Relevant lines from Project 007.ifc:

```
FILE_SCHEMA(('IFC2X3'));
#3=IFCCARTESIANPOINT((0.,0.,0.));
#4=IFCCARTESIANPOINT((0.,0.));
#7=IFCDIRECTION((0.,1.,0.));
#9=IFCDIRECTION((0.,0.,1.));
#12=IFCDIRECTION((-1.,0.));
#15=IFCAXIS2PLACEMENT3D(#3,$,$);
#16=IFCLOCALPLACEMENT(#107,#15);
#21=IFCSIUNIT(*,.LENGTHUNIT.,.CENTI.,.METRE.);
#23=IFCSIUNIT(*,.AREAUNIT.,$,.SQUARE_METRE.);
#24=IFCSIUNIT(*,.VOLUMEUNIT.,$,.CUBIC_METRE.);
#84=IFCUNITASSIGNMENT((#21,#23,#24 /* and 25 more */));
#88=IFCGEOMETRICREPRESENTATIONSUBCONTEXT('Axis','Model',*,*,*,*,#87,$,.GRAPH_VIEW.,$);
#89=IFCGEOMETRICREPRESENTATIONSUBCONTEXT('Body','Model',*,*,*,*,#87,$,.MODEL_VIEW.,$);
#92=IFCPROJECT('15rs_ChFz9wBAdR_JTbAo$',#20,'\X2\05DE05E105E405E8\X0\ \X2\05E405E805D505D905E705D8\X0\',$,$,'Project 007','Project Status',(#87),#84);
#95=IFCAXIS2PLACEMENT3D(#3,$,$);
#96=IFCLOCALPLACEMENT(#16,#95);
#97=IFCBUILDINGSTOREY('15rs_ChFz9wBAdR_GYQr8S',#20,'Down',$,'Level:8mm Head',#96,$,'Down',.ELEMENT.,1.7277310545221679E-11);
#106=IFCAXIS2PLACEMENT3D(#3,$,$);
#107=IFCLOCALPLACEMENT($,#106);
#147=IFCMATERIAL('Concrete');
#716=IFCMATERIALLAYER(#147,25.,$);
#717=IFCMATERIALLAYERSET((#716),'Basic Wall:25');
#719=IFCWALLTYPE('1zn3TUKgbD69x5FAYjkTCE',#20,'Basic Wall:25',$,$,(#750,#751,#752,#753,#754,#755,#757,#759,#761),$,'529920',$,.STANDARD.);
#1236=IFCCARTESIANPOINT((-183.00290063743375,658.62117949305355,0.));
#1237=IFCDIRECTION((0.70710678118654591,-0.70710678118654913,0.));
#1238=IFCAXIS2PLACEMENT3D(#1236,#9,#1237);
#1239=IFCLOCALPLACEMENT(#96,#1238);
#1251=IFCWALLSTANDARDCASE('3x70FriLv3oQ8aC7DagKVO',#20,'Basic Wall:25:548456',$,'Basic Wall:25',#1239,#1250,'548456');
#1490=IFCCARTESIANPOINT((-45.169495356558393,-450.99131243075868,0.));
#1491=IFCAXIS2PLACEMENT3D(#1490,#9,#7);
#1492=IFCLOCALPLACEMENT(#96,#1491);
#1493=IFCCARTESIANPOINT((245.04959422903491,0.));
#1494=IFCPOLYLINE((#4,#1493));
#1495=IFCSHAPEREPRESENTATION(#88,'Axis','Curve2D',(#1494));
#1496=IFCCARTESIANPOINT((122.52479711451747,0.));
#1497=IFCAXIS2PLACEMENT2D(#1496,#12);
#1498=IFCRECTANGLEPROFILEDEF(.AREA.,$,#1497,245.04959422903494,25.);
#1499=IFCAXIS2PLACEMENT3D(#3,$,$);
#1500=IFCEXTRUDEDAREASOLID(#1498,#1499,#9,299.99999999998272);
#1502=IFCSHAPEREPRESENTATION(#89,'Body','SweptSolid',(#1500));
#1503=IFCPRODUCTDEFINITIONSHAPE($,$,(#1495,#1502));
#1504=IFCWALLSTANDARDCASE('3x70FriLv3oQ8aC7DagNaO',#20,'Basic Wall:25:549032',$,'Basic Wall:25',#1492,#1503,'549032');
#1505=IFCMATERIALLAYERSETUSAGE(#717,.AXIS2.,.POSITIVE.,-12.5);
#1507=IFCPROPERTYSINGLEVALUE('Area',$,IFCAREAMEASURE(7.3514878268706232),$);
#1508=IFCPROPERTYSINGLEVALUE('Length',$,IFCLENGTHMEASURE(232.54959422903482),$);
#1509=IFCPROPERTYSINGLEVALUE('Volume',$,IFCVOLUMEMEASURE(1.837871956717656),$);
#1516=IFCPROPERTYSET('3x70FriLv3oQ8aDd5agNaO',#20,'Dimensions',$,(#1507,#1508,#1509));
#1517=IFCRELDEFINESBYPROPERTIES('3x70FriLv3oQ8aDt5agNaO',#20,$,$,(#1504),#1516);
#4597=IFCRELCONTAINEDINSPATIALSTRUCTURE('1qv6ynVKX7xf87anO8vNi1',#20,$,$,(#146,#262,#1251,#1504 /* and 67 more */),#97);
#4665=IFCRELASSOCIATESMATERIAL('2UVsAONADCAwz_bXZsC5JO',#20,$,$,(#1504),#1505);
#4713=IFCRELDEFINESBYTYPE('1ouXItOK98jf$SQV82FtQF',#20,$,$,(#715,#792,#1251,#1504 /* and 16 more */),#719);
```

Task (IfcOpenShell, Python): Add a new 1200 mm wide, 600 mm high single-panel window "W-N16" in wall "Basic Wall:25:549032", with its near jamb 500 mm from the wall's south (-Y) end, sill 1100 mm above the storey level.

```python
import numpy as np
import ifcopenshell
import ifcopenshell.api.feature
import ifcopenshell.api.geometry
import ifcopenshell.api.pset
import ifcopenshell.api.root
import ifcopenshell.api.spatial
import ifcopenshell.api.type
import ifcopenshell.geom
import ifcopenshell.util.element
import ifcopenshell.util.placement
import ifcopenshell.util.representation
import ifcopenshell.util.shape
import ifcopenshell.util.unit

model = ifcopenshell.open("Project 007.ifc")
unit_scale = ifcopenshell.util.unit.calculate_unit_scale(model)
area_scale = ifcopenshell.util.unit.calculate_unit_scale(model, "AREAUNIT")
volume_scale = ifcopenshell.util.unit.calculate_unit_scale(model, "VOLUMEUNIT")
settings = ifcopenshell.geom.settings()


def volume(element):
    """Net volume in cubic metres, openings subtracted."""
    shape = ifcopenshell.geom.create_shape(settings, element)
    return ifcopenshell.util.shape.get_volume(shape.geometry)


wall = model.by_guid("3x70FriLv3oQ8aC7DagNaO")
storey = ifcopenshell.util.element.get_container(wall, ifc_class="IfcBuildingStorey")
context = ifcopenshell.util.representation.get_context(model, "Model", "Body", "MODEL_VIEW")
before = volume(wall)

width, height, from_end, sill = 1.2, 0.6, 0.5, 1.1  # metres

# The wall runs along its own X axis, and the end named is its -X end.
wall_shape = ifcopenshell.geom.create_shape(settings, wall)
x, y, z = ifcopenshell.util.shape.get_vertices(wall_shape.geometry).T
start = x.min() + from_end
face, thickness = float(y.min()), float(y.max() - y.min())
wall_matrix = ifcopenshell.util.placement.get_local_placement(wall.ObjectPlacement)
level = ifcopenshell.util.placement.get_local_placement(storey.ObjectPlacement)[2, 3]


def in_wall(x, y):
    """Placement at x, y metres in the wall's axes, at sill height."""
    matrix = wall_matrix.copy()
    matrix[:, 3] = wall_matrix @ np.array([x / unit_scale, y / unit_scale, 0.0, 1.0])
    matrix[2, 3] = level + sill / unit_scale
    return matrix


# Opening: a box that overshoots both wall faces by 50 mm.
opening = ifcopenshell.api.root.create_entity(model, ifc_class="IfcOpeningElement")
box = ifcopenshell.api.geometry.add_wall_representation(
    model, context=context, length=width, height=height, thickness=thickness + 0.1
)
ifcopenshell.api.geometry.assign_representation(model, product=opening, representation=box)
ifcopenshell.api.geometry.edit_object_placement(model, product=opening, matrix=in_wall(start, face - 0.05), is_si=False)
ifcopenshell.api.feature.add_feature(model, feature=opening, element=wall)

window = ifcopenshell.api.root.create_entity(model, ifc_class="IfcWindow", name="W-N16")
window.OverallWidth, window.OverallHeight = width / unit_scale, height / unit_scale
body = ifcopenshell.api.geometry.add_window_representation(
    model,
    context=context,
    overall_width=window.OverallWidth,
    overall_height=window.OverallHeight,
    partition_type="SINGLE_PANEL",
)
ifcopenshell.api.geometry.assign_representation(model, product=window, representation=body)
ifcopenshell.api.spatial.assign_container(model, products=[window], relating_structure=storey)
fills = ifcopenshell.api.feature.add_filling(model, opening=opening, element=window)
fills.OwnerHistory = window.OwnerHistory  # required in IFC2X3

# IFC2X3 keeps the operation on the window style.
style = ifcopenshell.api.root.create_entity(model, ifc_class="IfcWindowStyle", name="W-N16")
style.OperationType, style.ConstructionType = "SINGLE_PANEL", "NOTDEFINED"
style.ParameterTakesPrecedence = style.Sizeable = False
ifcopenshell.api.type.assign_type(model, related_objects=[window], relating_type=style)

# Centre the window in the wall's thickness.
ifcopenshell.api.geometry.edit_object_placement(model, product=window, matrix=in_wall(start, face), is_si=False)
window_shape = ifcopenshell.geom.create_shape(settings, window)
depth = ifcopenshell.util.shape.get_vertices(window_shape.geometry)[:, 1]
offset = face + thickness / 2 - (depth.min() + depth.max()) / 2
ifcopenshell.api.geometry.edit_object_placement(model, product=window, matrix=in_wall(start, offset), is_si=False)

after = volume(wall)

# Update the wall's stored quantities.
pset = model.by_id(ifcopenshell.util.element.get_pset(wall, "Dimensions", should_inherit=False)["id"])
ifcopenshell.api.pset.edit_pset(model, pset=pset, properties={
    "Area": model.create_entity("IfcAreaMeasure", after / thickness / area_scale),
    "Volume": model.create_entity("IfcVolumeMeasure", after / volume_scale),
})

print(f"wall volume {before:.3f} -> {after:.3f} m3")

model.write("Project 007-out.ifc")
```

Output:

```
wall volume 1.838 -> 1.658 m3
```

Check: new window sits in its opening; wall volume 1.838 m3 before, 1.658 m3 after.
